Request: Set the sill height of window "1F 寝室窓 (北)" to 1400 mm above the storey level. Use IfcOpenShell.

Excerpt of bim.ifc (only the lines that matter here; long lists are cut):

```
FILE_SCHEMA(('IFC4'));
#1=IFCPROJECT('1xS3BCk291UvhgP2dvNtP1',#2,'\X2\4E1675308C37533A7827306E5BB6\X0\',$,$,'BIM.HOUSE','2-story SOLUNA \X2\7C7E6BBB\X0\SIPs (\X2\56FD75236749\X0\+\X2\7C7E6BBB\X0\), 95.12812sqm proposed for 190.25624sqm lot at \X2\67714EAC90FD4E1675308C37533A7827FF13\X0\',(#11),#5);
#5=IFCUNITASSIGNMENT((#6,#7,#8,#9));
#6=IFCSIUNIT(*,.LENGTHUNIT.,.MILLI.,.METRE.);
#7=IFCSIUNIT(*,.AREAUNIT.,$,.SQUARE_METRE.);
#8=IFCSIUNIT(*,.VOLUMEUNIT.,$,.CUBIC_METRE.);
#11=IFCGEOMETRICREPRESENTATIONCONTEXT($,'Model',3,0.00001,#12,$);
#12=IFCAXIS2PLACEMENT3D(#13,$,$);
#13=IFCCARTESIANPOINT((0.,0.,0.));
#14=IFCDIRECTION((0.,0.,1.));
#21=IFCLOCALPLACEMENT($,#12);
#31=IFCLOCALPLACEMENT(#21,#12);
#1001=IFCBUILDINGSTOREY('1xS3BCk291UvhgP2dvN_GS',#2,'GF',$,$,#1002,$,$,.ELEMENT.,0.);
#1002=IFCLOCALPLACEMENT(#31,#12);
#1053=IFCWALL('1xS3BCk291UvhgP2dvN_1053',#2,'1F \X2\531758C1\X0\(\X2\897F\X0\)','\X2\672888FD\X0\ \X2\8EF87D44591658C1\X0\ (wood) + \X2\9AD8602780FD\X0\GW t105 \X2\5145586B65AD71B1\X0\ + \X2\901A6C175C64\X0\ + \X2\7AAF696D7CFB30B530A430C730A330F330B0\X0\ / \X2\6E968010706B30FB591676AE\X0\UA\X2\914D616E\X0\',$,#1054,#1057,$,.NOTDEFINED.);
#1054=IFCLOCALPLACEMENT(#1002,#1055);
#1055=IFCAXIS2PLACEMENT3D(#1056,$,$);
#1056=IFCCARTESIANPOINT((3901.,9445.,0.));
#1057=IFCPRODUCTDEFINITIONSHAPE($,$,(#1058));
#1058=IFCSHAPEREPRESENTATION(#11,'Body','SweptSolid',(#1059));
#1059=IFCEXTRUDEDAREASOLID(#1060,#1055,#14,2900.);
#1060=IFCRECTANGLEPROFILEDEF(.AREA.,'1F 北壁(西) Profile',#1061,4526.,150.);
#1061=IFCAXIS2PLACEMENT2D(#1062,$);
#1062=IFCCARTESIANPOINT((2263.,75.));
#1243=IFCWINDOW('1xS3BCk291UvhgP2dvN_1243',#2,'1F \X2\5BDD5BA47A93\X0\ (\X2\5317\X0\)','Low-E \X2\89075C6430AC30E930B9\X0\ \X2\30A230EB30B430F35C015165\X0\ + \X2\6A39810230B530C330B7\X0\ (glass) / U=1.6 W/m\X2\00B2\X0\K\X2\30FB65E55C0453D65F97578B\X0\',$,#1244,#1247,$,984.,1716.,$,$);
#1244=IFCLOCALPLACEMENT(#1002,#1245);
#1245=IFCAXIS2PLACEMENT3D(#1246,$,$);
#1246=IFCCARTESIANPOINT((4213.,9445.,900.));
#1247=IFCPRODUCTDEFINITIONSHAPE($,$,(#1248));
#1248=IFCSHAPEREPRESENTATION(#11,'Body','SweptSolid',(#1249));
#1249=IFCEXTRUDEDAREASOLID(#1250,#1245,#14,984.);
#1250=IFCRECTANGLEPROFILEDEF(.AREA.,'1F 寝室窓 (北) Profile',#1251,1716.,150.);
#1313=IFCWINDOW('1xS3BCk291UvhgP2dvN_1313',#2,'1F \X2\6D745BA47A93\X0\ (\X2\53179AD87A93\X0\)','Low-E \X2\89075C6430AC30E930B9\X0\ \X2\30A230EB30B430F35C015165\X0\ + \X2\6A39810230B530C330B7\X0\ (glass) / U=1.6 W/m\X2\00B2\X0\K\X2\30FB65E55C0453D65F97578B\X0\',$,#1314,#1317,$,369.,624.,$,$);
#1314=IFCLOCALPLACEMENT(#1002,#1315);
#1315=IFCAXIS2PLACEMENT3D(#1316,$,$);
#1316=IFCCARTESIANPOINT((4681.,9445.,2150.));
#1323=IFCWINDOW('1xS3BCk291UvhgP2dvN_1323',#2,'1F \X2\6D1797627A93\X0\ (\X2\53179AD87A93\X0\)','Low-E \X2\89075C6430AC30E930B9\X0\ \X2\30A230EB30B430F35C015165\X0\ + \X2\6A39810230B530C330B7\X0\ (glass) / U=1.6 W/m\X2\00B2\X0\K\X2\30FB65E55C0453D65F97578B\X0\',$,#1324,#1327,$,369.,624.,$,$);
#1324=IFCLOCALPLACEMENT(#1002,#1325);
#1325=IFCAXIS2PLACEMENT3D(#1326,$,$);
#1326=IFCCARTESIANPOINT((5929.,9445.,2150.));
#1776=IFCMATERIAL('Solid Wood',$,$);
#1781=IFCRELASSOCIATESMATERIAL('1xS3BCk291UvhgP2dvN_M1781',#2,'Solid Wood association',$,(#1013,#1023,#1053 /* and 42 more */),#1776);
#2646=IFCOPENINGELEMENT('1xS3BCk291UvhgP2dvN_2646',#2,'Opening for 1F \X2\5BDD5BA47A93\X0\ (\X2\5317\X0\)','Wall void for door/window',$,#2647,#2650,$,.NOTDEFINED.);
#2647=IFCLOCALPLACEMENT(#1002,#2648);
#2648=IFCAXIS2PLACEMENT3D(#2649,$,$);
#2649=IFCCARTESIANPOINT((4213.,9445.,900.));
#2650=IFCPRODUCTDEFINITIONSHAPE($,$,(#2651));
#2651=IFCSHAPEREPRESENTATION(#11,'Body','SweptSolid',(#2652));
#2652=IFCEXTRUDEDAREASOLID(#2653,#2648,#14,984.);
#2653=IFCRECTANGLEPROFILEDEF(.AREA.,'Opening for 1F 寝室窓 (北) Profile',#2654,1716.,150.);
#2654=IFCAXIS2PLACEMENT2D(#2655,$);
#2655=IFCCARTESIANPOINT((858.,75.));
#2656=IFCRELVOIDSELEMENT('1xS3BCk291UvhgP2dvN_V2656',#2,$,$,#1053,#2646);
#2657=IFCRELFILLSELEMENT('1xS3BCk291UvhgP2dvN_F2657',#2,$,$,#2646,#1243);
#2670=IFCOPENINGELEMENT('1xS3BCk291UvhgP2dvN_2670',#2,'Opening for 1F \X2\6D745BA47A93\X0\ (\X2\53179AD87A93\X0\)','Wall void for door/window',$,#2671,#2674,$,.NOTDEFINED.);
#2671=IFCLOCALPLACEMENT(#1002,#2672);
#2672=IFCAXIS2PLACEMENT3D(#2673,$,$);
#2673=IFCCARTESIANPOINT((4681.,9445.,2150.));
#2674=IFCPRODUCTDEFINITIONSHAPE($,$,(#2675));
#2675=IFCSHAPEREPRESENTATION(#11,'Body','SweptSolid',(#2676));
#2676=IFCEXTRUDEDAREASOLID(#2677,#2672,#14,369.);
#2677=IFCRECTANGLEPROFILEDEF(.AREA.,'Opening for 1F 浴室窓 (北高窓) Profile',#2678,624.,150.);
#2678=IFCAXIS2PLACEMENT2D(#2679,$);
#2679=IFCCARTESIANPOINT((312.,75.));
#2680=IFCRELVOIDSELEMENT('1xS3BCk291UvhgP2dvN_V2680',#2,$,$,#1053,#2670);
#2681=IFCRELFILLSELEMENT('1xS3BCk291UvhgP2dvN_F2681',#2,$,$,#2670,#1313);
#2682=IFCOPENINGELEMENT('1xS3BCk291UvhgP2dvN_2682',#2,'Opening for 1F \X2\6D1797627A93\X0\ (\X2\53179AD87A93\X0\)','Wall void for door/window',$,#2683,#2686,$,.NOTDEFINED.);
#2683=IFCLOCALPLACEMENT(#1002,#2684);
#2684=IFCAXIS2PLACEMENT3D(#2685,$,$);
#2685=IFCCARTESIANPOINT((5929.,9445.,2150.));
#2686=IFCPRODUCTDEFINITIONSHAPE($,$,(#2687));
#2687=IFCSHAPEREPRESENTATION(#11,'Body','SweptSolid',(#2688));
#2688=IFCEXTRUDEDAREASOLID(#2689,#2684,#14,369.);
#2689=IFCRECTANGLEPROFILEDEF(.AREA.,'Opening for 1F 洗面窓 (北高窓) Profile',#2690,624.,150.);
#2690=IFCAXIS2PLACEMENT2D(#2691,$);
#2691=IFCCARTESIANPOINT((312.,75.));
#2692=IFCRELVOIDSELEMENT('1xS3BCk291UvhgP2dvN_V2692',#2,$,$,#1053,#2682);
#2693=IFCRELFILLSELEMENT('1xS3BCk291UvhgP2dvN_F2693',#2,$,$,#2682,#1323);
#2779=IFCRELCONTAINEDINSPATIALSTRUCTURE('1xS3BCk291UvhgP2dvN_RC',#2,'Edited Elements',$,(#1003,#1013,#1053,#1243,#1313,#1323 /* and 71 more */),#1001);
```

```python
import numpy as np
import ifcopenshell
import ifcopenshell.api.geometry
import ifcopenshell.geom
import ifcopenshell.util.element
import ifcopenshell.util.placement
import ifcopenshell.util.shape
import ifcopenshell.util.unit

model = ifcopenshell.open("bim.ifc")
unit_scale = ifcopenshell.util.unit.calculate_unit_scale(model)

window = model.by_guid("1xS3BCk291UvhgP2dvN_1243")
opening = window.FillsVoids[0].RelatingOpeningElement
storey = ifcopenshell.util.element.get_container(window, ifc_class="IfcBuildingStorey")
level = ifcopenshell.util.placement.get_local_placement(storey.ObjectPlacement)[2, 3]

# The opening's origin need not be at the sill, so measure its lowest point.
shape = ifcopenshell.geom.create_shape(ifcopenshell.geom.settings(), opening)
bottom = ifcopenshell.util.shape.get_shape_bottom_elevation(shape, shape.geometry) / unit_scale
dz = level + 1400.0 - bottom

shift = np.array([0.0, 0.0, dz])
# The window is not placed relative to its opening, so move both.
for product in (opening, window):
    matrix = ifcopenshell.util.placement.get_local_placement(product.ObjectPlacement)
    matrix[:3, 3] += shift
    ifcopenshell.api.geometry.edit_object_placement(model, product=product, matrix=matrix, is_si=False)

print(f"moved by {dz * unit_scale:+.3f} m")

model.write("bim-out.ifc")
```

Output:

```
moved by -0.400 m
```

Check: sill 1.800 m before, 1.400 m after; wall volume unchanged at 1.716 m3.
